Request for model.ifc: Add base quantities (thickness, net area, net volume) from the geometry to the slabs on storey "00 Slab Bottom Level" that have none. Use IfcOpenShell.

First a look at what the model holds.

```python
import ifcopenshell
import ifcopenshell.util.element
import ifcopenshell.util.unit

model = ifcopenshell.open("model.ifc")
print(model.schema)
for unit_type in ("LENGTHUNIT", "AREAUNIT", "VOLUMEUNIT"):
    print(unit_type, ifcopenshell.util.unit.calculate_unit_scale(model, unit_type))
storey = next(s for s in model.by_type("IfcBuildingStorey") if s.Name == "00 Slab Bottom Level")
slabs = [e for e in ifcopenshell.util.element.get_decomposition(storey) if e.is_a("IfcSlab")]
for e in sorted(slabs, key=lambda e: e.id()):
    print(e.id(), e.is_a(), e.Name, list(ifcopenshell.util.element.get_psets(e, qtos_only=True)), sep=" | ")
```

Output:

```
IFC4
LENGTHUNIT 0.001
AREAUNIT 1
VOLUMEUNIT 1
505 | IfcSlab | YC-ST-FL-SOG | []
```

```python
import ifcopenshell
import ifcopenshell.api.pset
import ifcopenshell.geom
import ifcopenshell.util.element
import ifcopenshell.util.shape
import ifcopenshell.util.unit

model = ifcopenshell.open("model.ifc")
unit_scale = ifcopenshell.util.unit.calculate_unit_scale(model)
area_scale = ifcopenshell.util.unit.calculate_unit_scale(model, "AREAUNIT")
volume_scale = ifcopenshell.util.unit.calculate_unit_scale(model, "VOLUMEUNIT")
settings = ifcopenshell.geom.settings()

storey = next(s for s in model.by_type("IfcBuildingStorey") if s.Name == "00 Slab Bottom Level")
slabs = [e for e in ifcopenshell.util.element.get_decomposition(storey) if e.is_a("IfcSlab")]

for e in sorted(slabs, key=lambda e: e.id()):
    if ifcopenshell.util.element.get_psets(e, qtos_only=True, should_inherit=False):
        continue
    # Geometry comes back in metres, in the element's own axes.
    shape = ifcopenshell.geom.create_shape(settings, e)
    values = {
        "Width": ifcopenshell.util.shape.get_z(shape.geometry) / unit_scale,
        "NetArea": ifcopenshell.util.shape.get_footprint_area(shape.geometry) / area_scale,
        "NetVolume": ifcopenshell.util.shape.get_volume(shape.geometry) / volume_scale,
    }
    qto = ifcopenshell.api.pset.add_qto(model, product=e, name="Qto_SlabBaseQuantities")
    ifcopenshell.api.pset.edit_qto(model, qto=qto, properties=values)
    print(e.id(), {k: round(v, 3) for k, v in values.items()})

model.write("model_v2.ifc")
```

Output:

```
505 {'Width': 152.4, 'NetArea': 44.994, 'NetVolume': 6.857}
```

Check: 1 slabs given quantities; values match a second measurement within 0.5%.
